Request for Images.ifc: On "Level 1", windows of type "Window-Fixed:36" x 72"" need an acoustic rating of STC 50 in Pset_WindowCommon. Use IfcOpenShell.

First a look at what the model holds.

```python
import ifcopenshell
import ifcopenshell.util.element

model = ifcopenshell.open("Images.ifc")
print(model.schema)
storey = next(s for s in model.by_type("IfcBuildingStorey") if s.Name == "Level 1")
windows = [e for e in ifcopenshell.util.element.get_decomposition(storey) if e.is_a("IfcWindow")]
seen = {}
for e in windows:
    element_type = ifcopenshell.util.element.get_type(e)
    key = (element_type.Name if element_type != e and element_type else None, ifcopenshell.util.element.get_pset(e, "Pset_WindowCommon", "AcousticRating"))
    seen[key] = seen.get(key, 0) + 1
for (name, value), count in sorted(seen.items(), key=str):
    print(count, "x", name, "|", value)
```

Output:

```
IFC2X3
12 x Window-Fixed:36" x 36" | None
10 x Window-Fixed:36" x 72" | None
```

```python
import ifcopenshell
import ifcopenshell.api.pset
import ifcopenshell.util.element

model = ifcopenshell.open("Images.ifc")

storey = next(s for s in model.by_type("IfcBuildingStorey") if s.Name == "Level 1")
windows = [e for e in ifcopenshell.util.element.get_decomposition(storey) if e.is_a("IfcWindow")]

count = 0
for e in windows:
    element_type = ifcopenshell.util.element.get_type(e)
    if element_type in (None, e) or element_type.Name != 'Window-Fixed:36" x 72"':
        continue
    # add_pset returns the element's existing set when there is one.
    pset = ifcopenshell.api.pset.add_pset(model, product=e, name="Pset_WindowCommon")
    ifcopenshell.api.pset.edit_pset(model, pset=pset, properties={"AcousticRating": "STC 50"})
    count += 1

print(count, "windows updated")

model.write("Images_edited.ifc")
```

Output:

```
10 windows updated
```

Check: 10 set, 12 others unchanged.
